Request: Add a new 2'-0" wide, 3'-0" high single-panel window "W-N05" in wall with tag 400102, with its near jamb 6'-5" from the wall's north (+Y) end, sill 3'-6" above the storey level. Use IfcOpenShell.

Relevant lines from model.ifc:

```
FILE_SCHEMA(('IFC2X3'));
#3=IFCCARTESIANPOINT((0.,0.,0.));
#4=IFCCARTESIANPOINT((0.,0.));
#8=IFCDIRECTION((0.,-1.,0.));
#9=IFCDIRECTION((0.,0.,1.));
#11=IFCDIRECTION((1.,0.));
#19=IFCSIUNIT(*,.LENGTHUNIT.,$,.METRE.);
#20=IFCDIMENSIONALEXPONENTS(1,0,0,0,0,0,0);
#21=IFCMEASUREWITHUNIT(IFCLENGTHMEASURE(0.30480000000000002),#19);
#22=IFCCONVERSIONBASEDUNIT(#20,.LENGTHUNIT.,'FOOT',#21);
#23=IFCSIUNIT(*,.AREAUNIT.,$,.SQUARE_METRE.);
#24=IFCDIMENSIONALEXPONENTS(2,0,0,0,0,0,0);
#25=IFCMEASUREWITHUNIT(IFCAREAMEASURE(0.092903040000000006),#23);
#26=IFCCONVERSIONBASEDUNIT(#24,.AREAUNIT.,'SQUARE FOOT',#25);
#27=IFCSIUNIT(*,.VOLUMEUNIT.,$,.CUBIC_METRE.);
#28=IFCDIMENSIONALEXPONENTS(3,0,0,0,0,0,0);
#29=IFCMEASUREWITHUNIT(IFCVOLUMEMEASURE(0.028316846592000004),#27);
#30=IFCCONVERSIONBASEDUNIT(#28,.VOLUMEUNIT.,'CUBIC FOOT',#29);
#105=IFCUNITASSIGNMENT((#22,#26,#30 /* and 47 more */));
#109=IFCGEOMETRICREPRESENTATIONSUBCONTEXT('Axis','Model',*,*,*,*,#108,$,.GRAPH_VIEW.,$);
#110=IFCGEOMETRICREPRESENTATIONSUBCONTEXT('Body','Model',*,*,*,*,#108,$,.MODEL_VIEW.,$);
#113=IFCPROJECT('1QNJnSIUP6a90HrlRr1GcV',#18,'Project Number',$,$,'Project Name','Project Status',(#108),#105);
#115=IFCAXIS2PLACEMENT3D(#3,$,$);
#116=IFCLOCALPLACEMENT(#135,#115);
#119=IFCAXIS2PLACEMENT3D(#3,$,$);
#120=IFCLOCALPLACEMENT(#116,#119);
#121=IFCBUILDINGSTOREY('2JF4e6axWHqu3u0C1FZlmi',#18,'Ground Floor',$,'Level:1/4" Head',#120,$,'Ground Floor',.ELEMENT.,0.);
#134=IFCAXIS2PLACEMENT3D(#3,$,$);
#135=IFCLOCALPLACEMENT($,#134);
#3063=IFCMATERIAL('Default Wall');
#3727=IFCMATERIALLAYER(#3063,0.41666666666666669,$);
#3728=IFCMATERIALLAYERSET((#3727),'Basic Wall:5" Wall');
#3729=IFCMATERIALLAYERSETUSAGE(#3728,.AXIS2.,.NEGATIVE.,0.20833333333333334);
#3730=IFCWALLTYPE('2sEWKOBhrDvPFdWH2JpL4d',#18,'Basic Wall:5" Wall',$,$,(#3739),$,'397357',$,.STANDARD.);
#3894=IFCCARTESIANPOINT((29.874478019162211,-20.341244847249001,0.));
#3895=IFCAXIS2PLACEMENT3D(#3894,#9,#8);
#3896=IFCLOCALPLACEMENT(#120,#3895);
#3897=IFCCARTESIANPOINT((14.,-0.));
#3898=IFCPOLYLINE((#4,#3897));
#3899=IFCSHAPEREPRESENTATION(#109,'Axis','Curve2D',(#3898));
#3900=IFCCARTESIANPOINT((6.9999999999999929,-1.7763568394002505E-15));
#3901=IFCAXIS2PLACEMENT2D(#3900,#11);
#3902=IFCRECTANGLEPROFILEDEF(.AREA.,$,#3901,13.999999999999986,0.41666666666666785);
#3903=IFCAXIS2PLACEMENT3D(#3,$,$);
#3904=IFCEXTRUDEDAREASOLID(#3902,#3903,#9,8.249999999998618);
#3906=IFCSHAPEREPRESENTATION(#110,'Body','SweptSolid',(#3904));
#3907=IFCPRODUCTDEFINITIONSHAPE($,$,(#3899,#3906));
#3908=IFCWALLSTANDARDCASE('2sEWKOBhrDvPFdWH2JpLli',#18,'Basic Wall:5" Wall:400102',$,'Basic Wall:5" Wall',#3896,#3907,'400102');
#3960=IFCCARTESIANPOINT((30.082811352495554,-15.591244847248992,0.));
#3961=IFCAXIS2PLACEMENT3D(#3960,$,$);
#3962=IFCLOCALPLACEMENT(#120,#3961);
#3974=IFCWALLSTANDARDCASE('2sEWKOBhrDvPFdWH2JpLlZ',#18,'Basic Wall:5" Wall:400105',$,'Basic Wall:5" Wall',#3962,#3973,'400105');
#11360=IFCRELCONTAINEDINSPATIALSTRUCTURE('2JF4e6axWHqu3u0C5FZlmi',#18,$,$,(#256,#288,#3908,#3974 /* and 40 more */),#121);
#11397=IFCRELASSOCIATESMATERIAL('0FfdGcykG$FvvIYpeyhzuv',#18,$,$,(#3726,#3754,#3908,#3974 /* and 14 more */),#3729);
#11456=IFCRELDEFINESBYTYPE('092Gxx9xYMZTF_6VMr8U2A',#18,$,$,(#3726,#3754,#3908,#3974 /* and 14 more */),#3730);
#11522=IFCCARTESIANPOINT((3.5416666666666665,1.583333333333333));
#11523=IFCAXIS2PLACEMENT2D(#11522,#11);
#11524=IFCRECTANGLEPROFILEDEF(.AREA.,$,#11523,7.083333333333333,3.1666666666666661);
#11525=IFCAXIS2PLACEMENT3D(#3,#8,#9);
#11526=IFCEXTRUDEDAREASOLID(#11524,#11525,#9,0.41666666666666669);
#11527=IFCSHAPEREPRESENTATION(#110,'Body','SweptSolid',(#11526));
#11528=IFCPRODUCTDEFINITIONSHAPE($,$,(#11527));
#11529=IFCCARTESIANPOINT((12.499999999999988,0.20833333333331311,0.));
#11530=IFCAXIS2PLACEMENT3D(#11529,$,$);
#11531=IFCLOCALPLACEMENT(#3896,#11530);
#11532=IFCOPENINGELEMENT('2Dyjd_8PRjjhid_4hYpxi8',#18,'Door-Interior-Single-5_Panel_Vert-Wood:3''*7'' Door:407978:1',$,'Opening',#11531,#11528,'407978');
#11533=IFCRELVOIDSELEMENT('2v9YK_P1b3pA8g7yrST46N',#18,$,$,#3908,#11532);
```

```python
import numpy as np
import ifcopenshell
import ifcopenshell.api.feature
import ifcopenshell.api.geometry
import ifcopenshell.api.root
import ifcopenshell.api.spatial
import ifcopenshell.api.type
import ifcopenshell.geom
import ifcopenshell.util.element
import ifcopenshell.util.placement
import ifcopenshell.util.representation
import ifcopenshell.util.shape
import ifcopenshell.util.unit

model = ifcopenshell.open("model.ifc")
unit_scale = ifcopenshell.util.unit.calculate_unit_scale(model)
settings = ifcopenshell.geom.settings()


def volume(element):
    """Net volume in cubic metres, openings subtracted."""
    shape = ifcopenshell.geom.create_shape(settings, element)
    return ifcopenshell.util.shape.get_volume(shape.geometry)


wall = model.by_guid("2sEWKOBhrDvPFdWH2JpLli")
storey = ifcopenshell.util.element.get_container(wall, ifc_class="IfcBuildingStorey")
context = ifcopenshell.util.representation.get_context(model, "Model", "Body", "MODEL_VIEW")
before = volume(wall)

width, height, from_end, sill = 0.6096, 0.9144, 1.9558, 1.0668  # metres

# The wall runs along its own X axis, and the end named is its -X end.
wall_shape = ifcopenshell.geom.create_shape(settings, wall)
x, y, z = ifcopenshell.util.shape.get_vertices(wall_shape.geometry).T
start = x.min() + from_end
face, thickness = float(y.min()), float(y.max() - y.min())
wall_matrix = ifcopenshell.util.placement.get_local_placement(wall.ObjectPlacement)
level = ifcopenshell.util.placement.get_local_placement(storey.ObjectPlacement)[2, 3]


def in_wall(x, y):
    """Placement at x, y metres in the wall's axes, at sill height."""
    matrix = wall_matrix.copy()
    matrix[:, 3] = wall_matrix @ np.array([x / unit_scale, y / unit_scale, 0.0, 1.0])
    matrix[2, 3] = level + sill / unit_scale
    return matrix


# Opening: a box that overshoots both wall faces by 50 mm.
opening = ifcopenshell.api.root.create_entity(model, ifc_class="IfcOpeningElement")
box = ifcopenshell.api.geometry.add_wall_representation(
    model, context=context, length=width, height=height, thickness=thickness + 0.1
)
ifcopenshell.api.geometry.assign_representation(model, product=opening, representation=box)
ifcopenshell.api.geometry.edit_object_placement(model, product=opening, matrix=in_wall(start, face - 0.05), is_si=False)
ifcopenshell.api.feature.add_feature(model, feature=opening, element=wall)

window = ifcopenshell.api.root.create_entity(model, ifc_class="IfcWindow", name="W-N05")
window.OverallWidth, window.OverallHeight = width / unit_scale, height / unit_scale
body = ifcopenshell.api.geometry.add_window_representation(
    model,
    context=context,
    overall_width=window.OverallWidth,
    overall_height=window.OverallHeight,
    partition_type="SINGLE_PANEL",
)
ifcopenshell.api.geometry.assign_representation(model, product=window, representation=body)
ifcopenshell.api.spatial.assign_container(model, products=[window], relating_structure=storey)
fills = ifcopenshell.api.feature.add_filling(model, opening=opening, element=window)
fills.OwnerHistory = window.OwnerHistory  # required in IFC2X3

# IFC2X3 keeps the operation on the window style.
style = ifcopenshell.api.root.create_entity(model, ifc_class="IfcWindowStyle", name="W-N05")
style.OperationType, style.ConstructionType = "SINGLE_PANEL", "NOTDEFINED"
style.ParameterTakesPrecedence = style.Sizeable = False
ifcopenshell.api.type.assign_type(model, related_objects=[window], relating_type=style)

# Centre the window in the wall's thickness.
ifcopenshell.api.geometry.edit_object_placement(model, product=window, matrix=in_wall(start, face), is_si=False)
window_shape = ifcopenshell.geom.create_shape(settings, window)
depth = ifcopenshell.util.shape.get_vertices(window_shape.geometry)[:, 1]
offset = face + thickness / 2 - (depth.min() + depth.max()) / 2
ifcopenshell.api.geometry.edit_object_placement(model, product=window, matrix=in_wall(start, offset), is_si=False)

after = volume(wall)

print(f"wall volume {before:.3f} -> {after:.3f} m3")

model.write("model_updated.ifc")
```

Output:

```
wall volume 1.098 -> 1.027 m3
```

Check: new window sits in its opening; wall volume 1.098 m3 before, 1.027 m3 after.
